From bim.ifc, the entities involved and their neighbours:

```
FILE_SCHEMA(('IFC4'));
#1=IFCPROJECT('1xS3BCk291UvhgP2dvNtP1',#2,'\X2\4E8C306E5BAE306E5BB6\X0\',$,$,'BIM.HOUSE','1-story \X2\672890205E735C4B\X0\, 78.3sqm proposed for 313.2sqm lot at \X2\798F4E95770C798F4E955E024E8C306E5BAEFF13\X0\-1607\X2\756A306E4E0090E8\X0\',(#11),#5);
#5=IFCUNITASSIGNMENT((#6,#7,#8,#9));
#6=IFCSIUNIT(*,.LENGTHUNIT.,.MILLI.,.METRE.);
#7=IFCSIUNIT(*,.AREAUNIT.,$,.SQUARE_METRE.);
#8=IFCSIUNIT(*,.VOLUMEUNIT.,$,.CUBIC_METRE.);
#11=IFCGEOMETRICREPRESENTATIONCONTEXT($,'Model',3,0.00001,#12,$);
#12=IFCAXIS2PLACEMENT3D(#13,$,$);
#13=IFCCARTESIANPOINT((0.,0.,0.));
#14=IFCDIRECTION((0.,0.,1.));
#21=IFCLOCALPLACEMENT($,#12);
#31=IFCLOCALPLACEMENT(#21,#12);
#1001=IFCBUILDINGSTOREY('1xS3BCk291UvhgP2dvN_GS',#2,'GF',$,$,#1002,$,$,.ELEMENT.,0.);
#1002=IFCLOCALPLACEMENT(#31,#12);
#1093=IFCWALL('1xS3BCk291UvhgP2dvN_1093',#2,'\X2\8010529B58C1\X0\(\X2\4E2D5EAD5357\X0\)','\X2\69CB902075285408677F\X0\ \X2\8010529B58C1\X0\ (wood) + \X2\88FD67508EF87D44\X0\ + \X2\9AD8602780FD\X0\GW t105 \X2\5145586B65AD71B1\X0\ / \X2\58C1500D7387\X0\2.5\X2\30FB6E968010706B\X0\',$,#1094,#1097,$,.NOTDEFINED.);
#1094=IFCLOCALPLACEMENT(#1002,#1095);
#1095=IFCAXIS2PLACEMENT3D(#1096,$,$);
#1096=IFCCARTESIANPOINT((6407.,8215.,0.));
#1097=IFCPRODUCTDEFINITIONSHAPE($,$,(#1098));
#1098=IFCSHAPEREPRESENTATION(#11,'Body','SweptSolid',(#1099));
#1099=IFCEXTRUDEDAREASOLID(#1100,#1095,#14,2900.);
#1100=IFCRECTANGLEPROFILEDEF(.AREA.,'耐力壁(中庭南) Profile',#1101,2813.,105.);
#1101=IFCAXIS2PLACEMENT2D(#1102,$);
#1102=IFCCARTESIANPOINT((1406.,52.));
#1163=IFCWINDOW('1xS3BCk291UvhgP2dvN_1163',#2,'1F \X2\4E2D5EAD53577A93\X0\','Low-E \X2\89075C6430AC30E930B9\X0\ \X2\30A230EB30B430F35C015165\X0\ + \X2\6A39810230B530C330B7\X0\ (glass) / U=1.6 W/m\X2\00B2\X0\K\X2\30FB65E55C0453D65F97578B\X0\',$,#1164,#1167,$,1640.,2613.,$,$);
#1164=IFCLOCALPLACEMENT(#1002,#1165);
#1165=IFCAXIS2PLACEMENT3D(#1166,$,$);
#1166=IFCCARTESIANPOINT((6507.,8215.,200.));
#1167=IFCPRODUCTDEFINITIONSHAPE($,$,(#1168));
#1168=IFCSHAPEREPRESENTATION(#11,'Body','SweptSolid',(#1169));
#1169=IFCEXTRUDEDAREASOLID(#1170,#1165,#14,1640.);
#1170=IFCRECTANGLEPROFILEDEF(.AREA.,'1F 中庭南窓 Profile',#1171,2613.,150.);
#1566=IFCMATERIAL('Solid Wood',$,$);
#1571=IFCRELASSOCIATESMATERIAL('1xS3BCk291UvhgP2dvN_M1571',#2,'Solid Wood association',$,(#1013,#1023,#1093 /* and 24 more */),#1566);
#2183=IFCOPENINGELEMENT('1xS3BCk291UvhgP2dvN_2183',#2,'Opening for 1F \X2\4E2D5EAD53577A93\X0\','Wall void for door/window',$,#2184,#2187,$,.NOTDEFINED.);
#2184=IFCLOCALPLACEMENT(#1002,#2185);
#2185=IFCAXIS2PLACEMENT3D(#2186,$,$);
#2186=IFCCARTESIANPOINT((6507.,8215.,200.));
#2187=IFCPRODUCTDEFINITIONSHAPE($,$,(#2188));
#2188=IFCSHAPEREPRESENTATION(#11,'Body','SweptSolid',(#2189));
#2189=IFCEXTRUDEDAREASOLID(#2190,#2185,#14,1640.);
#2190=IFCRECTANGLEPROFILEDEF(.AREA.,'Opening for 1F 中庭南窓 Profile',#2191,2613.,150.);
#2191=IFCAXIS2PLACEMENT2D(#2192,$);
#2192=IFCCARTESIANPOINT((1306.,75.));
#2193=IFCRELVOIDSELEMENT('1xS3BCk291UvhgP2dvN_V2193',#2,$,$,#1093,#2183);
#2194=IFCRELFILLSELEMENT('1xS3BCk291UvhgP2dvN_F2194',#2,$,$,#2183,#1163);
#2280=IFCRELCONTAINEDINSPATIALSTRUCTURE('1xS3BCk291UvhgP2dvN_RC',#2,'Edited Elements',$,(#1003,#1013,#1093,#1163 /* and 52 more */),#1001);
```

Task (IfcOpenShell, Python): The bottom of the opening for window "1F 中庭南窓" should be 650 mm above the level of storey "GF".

```python
import numpy as np
import ifcopenshell
import ifcopenshell.api.geometry
import ifcopenshell.geom
import ifcopenshell.util.element
import ifcopenshell.util.placement
import ifcopenshell.util.shape
import ifcopenshell.util.unit

model = ifcopenshell.open("bim.ifc")
unit_scale = ifcopenshell.util.unit.calculate_unit_scale(model)

window = model.by_id(1163)
opening = window.FillsVoids[0].RelatingOpeningElement
storey = ifcopenshell.util.element.get_container(window, ifc_class="IfcBuildingStorey")
level = ifcopenshell.util.placement.get_local_placement(storey.ObjectPlacement)[2, 3]

# The opening's origin need not be at the sill, so measure its lowest point.
shape = ifcopenshell.geom.create_shape(ifcopenshell.geom.settings(), opening)
bottom = ifcopenshell.util.shape.get_shape_bottom_elevation(shape, shape.geometry) / unit_scale
dz = level + 650.0 - bottom

shift = np.array([0.0, 0.0, dz])
# The window is not placed relative to its opening, so move both.
for product in (opening, window):
    matrix = ifcopenshell.util.placement.get_local_placement(product.ObjectPlacement)
    matrix[:3, 3] += shift
    ifcopenshell.api.geometry.edit_object_placement(model, product=product, matrix=matrix, is_si=False)

print(f"moved by {dz * unit_scale:+.3f} m")

model.write("bim-out.ifc")
```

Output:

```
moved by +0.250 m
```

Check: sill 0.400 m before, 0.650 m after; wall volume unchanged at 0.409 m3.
